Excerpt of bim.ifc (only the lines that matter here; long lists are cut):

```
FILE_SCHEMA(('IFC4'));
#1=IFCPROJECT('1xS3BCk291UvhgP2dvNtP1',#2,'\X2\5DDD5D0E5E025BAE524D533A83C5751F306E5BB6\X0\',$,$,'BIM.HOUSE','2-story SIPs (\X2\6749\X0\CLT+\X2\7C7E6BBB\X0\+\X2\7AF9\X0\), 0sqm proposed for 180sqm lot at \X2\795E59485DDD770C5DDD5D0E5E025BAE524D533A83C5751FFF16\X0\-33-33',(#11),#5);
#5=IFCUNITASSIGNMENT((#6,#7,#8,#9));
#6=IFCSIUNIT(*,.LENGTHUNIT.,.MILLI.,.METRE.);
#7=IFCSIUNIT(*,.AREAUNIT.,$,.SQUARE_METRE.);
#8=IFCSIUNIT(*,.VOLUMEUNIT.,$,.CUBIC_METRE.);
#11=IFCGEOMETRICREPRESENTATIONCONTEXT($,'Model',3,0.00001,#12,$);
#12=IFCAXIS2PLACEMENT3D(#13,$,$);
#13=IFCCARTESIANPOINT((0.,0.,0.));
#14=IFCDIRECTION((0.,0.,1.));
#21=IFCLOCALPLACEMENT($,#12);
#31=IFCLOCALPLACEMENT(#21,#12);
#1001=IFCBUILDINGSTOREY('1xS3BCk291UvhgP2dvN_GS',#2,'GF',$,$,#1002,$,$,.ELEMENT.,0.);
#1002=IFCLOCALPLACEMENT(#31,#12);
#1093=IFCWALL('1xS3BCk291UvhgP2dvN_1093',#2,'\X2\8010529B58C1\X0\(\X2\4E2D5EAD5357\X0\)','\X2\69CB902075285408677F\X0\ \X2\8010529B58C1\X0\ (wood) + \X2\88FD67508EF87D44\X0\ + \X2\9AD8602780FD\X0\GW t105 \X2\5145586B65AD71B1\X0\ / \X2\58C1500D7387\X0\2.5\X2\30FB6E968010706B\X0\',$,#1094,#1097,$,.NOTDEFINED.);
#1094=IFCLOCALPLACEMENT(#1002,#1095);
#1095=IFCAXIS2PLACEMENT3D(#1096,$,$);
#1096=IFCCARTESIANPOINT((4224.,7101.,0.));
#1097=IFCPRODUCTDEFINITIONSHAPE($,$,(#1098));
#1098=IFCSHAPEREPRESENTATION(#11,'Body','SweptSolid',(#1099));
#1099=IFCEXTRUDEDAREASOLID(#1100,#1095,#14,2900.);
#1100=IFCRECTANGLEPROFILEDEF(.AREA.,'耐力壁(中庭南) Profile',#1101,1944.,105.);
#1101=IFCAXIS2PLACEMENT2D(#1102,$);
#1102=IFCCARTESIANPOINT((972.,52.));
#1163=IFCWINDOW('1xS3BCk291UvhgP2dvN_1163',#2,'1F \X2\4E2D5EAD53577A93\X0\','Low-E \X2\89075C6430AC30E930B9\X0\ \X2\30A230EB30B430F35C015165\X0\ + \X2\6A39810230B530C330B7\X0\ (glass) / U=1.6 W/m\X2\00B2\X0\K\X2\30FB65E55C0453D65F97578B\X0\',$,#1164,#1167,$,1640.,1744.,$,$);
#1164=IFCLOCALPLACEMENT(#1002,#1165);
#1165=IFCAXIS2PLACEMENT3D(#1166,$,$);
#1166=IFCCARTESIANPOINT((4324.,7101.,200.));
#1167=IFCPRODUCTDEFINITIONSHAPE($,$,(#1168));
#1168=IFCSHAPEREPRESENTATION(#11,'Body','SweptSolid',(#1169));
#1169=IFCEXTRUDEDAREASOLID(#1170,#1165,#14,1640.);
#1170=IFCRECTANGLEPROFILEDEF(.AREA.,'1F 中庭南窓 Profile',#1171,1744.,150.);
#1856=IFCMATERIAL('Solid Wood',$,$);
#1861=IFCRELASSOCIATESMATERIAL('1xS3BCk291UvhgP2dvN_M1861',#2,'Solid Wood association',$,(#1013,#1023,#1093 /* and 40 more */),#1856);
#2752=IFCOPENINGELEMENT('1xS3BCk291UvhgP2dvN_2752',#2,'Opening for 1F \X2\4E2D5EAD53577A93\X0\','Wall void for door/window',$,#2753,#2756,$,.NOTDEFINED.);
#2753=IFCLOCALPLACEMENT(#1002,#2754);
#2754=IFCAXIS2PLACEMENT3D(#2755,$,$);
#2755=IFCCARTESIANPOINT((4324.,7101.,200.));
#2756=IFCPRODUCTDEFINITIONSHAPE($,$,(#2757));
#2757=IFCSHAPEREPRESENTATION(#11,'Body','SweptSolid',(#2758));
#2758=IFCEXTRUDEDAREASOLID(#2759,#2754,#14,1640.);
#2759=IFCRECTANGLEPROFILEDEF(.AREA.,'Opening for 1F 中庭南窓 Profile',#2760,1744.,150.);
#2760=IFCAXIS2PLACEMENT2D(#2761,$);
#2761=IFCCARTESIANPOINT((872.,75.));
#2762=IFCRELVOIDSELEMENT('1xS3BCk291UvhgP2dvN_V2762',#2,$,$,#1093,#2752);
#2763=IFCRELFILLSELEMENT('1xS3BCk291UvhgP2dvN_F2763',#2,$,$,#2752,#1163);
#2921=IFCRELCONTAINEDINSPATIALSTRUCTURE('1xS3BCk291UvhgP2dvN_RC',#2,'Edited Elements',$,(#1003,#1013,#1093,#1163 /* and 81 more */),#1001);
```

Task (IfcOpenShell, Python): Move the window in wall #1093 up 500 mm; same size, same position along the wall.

```python
import numpy as np
import ifcopenshell
import ifcopenshell.api.geometry
import ifcopenshell.util.placement
import ifcopenshell.util.unit

model = ifcopenshell.open("bim.ifc")
unit_scale = ifcopenshell.util.unit.calculate_unit_scale(model)

window = model.by_guid("1xS3BCk291UvhgP2dvN_1163")
opening = window.FillsVoids[0].RelatingOpeningElement
dz = 0.5 / unit_scale

shift = np.array([0.0, 0.0, dz])
# The window is not placed relative to its opening, so move both.
for product in (opening, window):
    matrix = ifcopenshell.util.placement.get_local_placement(product.ObjectPlacement)
    matrix[:3, 3] += shift
    ifcopenshell.api.geometry.edit_object_placement(model, product=product, matrix=matrix, is_si=False)

print(f"moved by {dz * unit_scale:+.3f} m")

model.write("bim_rev.ifc")
```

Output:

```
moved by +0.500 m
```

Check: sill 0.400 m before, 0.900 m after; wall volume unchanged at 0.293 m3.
